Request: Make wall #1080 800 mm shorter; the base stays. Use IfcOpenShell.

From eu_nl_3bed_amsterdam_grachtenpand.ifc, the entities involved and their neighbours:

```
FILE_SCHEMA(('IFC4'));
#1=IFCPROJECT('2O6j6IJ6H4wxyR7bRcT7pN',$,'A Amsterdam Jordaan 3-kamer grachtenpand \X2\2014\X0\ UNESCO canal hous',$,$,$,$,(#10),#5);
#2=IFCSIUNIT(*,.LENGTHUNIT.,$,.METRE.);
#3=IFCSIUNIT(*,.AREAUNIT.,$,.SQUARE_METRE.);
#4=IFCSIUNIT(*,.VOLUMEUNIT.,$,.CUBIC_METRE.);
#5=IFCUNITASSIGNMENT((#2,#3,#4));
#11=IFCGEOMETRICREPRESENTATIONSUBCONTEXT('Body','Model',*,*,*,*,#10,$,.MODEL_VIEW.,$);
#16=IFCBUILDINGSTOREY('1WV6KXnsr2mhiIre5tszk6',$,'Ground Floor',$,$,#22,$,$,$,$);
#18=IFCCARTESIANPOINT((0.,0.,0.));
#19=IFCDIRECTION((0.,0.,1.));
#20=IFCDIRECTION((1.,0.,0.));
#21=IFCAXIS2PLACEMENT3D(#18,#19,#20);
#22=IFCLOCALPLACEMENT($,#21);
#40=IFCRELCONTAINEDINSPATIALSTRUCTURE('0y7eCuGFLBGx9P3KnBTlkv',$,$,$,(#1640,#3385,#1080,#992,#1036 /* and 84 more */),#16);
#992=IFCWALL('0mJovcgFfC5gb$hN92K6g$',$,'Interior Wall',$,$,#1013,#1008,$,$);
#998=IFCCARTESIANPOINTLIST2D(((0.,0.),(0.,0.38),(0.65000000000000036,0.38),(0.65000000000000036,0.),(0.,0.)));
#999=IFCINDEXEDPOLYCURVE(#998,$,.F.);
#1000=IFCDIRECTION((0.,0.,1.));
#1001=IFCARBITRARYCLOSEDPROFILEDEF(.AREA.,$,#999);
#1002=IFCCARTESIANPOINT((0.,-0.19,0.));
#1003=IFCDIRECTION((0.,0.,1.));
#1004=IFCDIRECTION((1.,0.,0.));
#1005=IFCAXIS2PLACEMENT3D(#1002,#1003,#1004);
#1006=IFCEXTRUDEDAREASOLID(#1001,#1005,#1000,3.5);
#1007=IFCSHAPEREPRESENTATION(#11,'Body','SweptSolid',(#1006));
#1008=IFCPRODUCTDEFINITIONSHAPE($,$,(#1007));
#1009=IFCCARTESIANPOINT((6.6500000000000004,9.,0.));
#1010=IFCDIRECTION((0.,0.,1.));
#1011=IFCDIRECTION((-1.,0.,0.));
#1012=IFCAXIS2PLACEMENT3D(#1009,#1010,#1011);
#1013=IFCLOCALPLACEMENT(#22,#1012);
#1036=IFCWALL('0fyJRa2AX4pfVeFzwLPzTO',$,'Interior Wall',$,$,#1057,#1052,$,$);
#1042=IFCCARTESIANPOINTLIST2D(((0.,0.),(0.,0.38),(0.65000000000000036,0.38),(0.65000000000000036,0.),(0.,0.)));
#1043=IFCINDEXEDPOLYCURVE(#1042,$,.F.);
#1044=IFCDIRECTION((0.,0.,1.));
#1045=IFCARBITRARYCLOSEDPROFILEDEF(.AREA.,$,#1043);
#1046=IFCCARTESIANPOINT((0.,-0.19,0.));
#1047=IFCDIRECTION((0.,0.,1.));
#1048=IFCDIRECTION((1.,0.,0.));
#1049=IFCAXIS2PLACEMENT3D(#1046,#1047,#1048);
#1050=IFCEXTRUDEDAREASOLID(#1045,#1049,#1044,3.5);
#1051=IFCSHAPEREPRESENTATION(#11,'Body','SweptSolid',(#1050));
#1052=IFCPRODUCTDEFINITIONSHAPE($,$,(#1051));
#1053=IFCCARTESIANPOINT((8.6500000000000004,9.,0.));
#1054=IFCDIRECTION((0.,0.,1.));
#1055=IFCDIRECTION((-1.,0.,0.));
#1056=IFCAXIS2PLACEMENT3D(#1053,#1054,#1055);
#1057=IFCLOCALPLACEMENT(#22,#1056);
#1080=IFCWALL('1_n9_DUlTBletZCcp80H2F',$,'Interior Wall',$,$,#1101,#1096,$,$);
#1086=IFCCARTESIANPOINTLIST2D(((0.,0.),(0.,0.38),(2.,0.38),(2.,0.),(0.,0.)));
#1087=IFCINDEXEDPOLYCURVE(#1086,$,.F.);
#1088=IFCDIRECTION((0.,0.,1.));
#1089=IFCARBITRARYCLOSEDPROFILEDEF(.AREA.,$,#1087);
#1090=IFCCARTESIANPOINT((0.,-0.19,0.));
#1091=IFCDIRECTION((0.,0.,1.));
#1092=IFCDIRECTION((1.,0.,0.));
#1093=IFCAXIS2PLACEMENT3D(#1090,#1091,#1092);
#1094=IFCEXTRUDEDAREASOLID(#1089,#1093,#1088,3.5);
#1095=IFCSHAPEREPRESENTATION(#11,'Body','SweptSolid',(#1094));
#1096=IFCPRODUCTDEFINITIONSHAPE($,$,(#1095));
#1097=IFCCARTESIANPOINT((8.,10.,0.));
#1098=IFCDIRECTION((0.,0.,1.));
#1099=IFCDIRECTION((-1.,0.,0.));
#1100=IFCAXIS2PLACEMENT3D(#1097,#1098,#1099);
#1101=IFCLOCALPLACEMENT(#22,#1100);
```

```python
import ifcopenshell
import ifcopenshell.geom
import ifcopenshell.util.representation
import ifcopenshell.util.shape
import ifcopenshell.util.unit

model = ifcopenshell.open("eu_nl_3bed_amsterdam_grachtenpand.ifc")
unit_scale = ifcopenshell.util.unit.calculate_unit_scale(model)
settings = ifcopenshell.geom.settings()


def volume(element):
    """Net volume in cubic metres, openings subtracted."""
    shape = ifcopenshell.geom.create_shape(settings, element)
    return ifcopenshell.util.shape.get_volume(shape.geometry)


wall = model.by_guid("1_n9_DUlTBletZCcp80H2F")
before = volume(wall)

body = ifcopenshell.util.representation.get_representation(wall, "Model", "Body")
solid = body.Items[0]
old_height = solid.Depth
solid.Depth -= 0.8 / unit_scale
after = volume(wall)

print(f"height {old_height:g} -> {solid.Depth:g}, volume {before:.3f} -> {after:.3f} m3")

model.write("eu_nl_3bed_amsterdam_grachtenpand_updated.ifc")
```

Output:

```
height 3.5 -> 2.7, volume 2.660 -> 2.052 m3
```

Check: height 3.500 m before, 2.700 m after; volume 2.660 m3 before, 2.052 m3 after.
